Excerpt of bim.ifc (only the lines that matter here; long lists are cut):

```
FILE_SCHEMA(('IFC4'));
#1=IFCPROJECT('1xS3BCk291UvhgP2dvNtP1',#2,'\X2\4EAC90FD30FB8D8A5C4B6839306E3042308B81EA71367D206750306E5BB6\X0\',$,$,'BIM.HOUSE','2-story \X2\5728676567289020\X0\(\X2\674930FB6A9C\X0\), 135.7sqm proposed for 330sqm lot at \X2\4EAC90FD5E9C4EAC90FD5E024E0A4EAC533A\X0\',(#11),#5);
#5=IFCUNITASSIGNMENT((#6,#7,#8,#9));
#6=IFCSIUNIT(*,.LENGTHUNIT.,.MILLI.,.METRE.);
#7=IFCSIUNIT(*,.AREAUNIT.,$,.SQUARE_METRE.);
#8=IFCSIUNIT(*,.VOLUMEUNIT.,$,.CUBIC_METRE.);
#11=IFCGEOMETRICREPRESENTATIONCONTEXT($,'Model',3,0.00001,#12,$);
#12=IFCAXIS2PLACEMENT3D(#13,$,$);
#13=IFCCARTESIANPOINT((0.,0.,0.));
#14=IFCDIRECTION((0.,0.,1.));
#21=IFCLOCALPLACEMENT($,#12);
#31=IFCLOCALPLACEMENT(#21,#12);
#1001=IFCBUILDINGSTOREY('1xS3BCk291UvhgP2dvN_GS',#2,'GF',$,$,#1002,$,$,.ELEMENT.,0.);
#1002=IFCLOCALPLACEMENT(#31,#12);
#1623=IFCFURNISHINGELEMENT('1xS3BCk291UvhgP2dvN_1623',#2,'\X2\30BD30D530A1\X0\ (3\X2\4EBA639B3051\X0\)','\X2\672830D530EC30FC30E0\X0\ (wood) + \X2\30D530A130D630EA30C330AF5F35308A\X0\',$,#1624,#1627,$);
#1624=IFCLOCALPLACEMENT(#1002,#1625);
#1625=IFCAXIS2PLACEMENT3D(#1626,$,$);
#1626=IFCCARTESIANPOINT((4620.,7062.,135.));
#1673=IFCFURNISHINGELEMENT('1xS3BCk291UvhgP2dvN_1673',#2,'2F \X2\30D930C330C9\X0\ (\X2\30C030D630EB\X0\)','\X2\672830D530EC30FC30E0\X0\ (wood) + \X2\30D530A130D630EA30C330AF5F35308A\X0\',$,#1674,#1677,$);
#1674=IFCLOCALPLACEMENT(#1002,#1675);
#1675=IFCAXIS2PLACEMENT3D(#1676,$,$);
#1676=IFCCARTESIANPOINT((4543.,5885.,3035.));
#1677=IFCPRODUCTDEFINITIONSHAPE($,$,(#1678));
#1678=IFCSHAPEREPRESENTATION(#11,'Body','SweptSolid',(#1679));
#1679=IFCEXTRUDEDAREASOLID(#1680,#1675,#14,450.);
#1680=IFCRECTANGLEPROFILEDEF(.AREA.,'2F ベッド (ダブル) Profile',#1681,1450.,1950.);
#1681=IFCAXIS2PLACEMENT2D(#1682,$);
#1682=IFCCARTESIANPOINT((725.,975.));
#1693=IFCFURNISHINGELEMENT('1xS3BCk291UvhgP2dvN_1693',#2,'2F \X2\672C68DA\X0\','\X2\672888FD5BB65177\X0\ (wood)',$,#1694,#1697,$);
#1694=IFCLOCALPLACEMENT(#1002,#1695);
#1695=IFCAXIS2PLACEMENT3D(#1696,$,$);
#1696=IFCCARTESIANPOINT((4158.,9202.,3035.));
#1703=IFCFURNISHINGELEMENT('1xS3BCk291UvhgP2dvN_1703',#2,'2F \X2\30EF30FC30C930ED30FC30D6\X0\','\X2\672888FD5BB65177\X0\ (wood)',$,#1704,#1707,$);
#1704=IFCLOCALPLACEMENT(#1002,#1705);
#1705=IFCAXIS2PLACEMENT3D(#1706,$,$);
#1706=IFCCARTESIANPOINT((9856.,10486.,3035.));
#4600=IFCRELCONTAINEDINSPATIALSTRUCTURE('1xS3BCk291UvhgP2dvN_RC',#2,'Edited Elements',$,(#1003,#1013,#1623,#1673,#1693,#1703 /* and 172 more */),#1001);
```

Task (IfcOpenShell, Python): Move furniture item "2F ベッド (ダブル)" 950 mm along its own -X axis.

```python
import ifcopenshell
import ifcopenshell.api.geometry
import ifcopenshell.util.placement
import ifcopenshell.util.unit

model = ifcopenshell.open("bim.ifc")
unit_scale = ifcopenshell.util.unit.calculate_unit_scale(model)

item = model.by_guid("1xS3BCk291UvhgP2dvN_1673")
matrix = ifcopenshell.util.placement.get_local_placement(item.ObjectPlacement)
matrix[:3, 3] -= matrix[:3, 0] * 0.95 / unit_scale
ifcopenshell.api.geometry.edit_object_placement(model, product=item, matrix=matrix, is_si=False)

print(ifcopenshell.util.placement.get_local_placement(item.ObjectPlacement).round(3) + 0.0)

model.write("bim_v2.ifc")
```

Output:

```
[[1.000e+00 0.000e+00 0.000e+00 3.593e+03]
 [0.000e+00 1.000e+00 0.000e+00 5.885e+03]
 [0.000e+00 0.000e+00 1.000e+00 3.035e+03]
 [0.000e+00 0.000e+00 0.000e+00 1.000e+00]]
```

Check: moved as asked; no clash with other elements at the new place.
